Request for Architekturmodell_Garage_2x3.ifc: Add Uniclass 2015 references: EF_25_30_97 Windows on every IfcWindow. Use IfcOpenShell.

First a look at what the model holds.

```python
import ifcopenshell

model = ifcopenshell.open("Architekturmodell_Garage_2x3.ifc")
print(model.schema)
print("classifications:", [c.Name for c in model.by_type("IfcClassification")])
for ifc_class in ("IfcDoor", "IfcRoof", "IfcStair", "IfcWall", "IfcWindow"):
    print(ifc_class, len(model.by_type(ifc_class)))
```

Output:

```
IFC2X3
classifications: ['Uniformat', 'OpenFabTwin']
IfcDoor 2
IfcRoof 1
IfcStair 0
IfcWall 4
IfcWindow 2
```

```python
import ifcopenshell
import ifcopenshell.api.classification

model = ifcopenshell.open("Architekturmodell_Garage_2x3.ifc")

# IFC2X3 requires Source and Edition and has no link from the project to the system.
system = model.create_entity("IfcClassification", Source="NBS", Edition="2015", Name="Uniclass 2015")

codes = {
    "IfcWindow": ("EF_25_30_97", "Windows"),
}
for ifc_class, (code, name) in codes.items():
    products = model.by_type(ifc_class)
    ifcopenshell.api.classification.add_reference(
        model, products=products, classification=system, identification=code, name=name
    )
    print(code, len(products))

model.write("Architekturmodell_Garage_2x3_rev.ifc")
```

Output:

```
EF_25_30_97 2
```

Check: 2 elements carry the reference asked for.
